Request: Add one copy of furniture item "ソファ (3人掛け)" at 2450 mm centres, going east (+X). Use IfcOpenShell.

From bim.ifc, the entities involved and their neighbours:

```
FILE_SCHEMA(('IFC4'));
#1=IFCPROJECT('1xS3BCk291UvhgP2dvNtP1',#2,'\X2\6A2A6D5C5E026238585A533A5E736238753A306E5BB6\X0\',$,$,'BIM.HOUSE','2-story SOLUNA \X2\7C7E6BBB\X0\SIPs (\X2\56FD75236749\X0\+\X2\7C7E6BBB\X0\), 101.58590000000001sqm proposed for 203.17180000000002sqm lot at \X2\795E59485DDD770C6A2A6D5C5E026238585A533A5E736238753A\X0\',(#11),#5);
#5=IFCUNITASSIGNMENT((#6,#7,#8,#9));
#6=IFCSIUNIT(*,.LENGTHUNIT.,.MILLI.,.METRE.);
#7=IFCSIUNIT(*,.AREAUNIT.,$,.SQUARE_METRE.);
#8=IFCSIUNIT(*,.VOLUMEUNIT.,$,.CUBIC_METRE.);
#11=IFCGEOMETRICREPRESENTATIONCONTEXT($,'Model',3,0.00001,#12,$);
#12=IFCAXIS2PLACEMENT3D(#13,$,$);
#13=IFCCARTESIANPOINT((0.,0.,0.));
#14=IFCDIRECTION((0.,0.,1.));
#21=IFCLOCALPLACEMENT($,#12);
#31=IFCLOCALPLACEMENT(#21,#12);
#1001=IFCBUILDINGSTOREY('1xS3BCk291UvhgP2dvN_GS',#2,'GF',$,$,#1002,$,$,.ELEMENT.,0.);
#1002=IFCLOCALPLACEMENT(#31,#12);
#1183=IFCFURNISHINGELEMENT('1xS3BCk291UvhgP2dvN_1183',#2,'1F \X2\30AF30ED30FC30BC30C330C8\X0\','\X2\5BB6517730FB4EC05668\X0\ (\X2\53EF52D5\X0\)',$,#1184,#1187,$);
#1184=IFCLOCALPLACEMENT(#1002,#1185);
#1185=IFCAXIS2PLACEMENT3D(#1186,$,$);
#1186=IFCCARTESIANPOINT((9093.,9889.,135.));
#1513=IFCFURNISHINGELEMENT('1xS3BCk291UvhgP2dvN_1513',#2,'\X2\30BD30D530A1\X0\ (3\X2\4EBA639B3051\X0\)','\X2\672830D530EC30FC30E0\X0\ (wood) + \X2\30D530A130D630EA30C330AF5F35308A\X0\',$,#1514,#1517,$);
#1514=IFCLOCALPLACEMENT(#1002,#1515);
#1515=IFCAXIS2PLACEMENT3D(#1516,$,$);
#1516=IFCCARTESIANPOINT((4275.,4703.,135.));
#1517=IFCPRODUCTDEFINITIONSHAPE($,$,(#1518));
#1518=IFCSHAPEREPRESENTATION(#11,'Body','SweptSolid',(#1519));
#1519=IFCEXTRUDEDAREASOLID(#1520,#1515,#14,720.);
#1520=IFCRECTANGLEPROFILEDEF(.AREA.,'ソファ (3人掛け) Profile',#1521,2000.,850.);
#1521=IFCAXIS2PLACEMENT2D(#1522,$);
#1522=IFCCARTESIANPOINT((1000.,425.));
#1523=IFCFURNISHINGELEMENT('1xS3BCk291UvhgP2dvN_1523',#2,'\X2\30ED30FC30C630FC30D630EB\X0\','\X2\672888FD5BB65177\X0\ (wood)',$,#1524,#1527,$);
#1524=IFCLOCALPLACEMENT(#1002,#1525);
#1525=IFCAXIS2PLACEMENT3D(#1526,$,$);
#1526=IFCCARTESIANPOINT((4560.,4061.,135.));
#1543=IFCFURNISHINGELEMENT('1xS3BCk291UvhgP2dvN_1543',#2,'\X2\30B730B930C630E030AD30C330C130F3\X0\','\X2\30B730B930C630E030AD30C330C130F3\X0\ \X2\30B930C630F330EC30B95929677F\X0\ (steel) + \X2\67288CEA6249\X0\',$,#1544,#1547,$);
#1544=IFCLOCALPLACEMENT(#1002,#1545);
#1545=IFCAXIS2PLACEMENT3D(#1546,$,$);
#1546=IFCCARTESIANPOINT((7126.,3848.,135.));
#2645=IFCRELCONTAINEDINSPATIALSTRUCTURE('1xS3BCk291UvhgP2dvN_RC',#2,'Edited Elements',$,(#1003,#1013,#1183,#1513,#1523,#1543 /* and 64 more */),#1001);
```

```python
import numpy as np
import ifcopenshell
import ifcopenshell.api.geometry
import ifcopenshell.api.root
import ifcopenshell.util.element
import ifcopenshell.util.placement

model = ifcopenshell.open("bim.ifc")


def reuse_history(source, copy):
    """copy_class also copies each property set's owner history, people and application; keep the originals."""
    for rel in copy.IsDefinedBy:
        if rel.is_a("IfcRelDefinesByProperties") and (history := rel.RelatingPropertyDefinition.OwnerHistory):
            rel.RelatingPropertyDefinition.OwnerHistory = source.OwnerHistory
            ifcopenshell.util.element.remove_deep2(model, history)


source = model.by_guid("1xS3BCk291UvhgP2dvN_1513")
base = ifcopenshell.util.placement.get_local_placement(source.ObjectPlacement)
step = np.array([1.0, 0.0, 0.0]) * 2450.0

for i in range(1, 2):
    copy = ifcopenshell.api.root.copy_class(model, product=source)
    copy.Representation = ifcopenshell.util.element.copy_deep(
        model, source.Representation, exclude=["IfcGeometricRepresentationContext", "IfcRepresentationMap"]
    )
    reuse_history(source, copy)
    matrix = base.copy()
    matrix[:3, 3] += i * step
    print("added at", matrix[:3, 3].round(3) + 0.0)
    ifcopenshell.api.geometry.edit_object_placement(model, product=copy, matrix=matrix, is_si=False)

model.write("bim_rev.ifc")
```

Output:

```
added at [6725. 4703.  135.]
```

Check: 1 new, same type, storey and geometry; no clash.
